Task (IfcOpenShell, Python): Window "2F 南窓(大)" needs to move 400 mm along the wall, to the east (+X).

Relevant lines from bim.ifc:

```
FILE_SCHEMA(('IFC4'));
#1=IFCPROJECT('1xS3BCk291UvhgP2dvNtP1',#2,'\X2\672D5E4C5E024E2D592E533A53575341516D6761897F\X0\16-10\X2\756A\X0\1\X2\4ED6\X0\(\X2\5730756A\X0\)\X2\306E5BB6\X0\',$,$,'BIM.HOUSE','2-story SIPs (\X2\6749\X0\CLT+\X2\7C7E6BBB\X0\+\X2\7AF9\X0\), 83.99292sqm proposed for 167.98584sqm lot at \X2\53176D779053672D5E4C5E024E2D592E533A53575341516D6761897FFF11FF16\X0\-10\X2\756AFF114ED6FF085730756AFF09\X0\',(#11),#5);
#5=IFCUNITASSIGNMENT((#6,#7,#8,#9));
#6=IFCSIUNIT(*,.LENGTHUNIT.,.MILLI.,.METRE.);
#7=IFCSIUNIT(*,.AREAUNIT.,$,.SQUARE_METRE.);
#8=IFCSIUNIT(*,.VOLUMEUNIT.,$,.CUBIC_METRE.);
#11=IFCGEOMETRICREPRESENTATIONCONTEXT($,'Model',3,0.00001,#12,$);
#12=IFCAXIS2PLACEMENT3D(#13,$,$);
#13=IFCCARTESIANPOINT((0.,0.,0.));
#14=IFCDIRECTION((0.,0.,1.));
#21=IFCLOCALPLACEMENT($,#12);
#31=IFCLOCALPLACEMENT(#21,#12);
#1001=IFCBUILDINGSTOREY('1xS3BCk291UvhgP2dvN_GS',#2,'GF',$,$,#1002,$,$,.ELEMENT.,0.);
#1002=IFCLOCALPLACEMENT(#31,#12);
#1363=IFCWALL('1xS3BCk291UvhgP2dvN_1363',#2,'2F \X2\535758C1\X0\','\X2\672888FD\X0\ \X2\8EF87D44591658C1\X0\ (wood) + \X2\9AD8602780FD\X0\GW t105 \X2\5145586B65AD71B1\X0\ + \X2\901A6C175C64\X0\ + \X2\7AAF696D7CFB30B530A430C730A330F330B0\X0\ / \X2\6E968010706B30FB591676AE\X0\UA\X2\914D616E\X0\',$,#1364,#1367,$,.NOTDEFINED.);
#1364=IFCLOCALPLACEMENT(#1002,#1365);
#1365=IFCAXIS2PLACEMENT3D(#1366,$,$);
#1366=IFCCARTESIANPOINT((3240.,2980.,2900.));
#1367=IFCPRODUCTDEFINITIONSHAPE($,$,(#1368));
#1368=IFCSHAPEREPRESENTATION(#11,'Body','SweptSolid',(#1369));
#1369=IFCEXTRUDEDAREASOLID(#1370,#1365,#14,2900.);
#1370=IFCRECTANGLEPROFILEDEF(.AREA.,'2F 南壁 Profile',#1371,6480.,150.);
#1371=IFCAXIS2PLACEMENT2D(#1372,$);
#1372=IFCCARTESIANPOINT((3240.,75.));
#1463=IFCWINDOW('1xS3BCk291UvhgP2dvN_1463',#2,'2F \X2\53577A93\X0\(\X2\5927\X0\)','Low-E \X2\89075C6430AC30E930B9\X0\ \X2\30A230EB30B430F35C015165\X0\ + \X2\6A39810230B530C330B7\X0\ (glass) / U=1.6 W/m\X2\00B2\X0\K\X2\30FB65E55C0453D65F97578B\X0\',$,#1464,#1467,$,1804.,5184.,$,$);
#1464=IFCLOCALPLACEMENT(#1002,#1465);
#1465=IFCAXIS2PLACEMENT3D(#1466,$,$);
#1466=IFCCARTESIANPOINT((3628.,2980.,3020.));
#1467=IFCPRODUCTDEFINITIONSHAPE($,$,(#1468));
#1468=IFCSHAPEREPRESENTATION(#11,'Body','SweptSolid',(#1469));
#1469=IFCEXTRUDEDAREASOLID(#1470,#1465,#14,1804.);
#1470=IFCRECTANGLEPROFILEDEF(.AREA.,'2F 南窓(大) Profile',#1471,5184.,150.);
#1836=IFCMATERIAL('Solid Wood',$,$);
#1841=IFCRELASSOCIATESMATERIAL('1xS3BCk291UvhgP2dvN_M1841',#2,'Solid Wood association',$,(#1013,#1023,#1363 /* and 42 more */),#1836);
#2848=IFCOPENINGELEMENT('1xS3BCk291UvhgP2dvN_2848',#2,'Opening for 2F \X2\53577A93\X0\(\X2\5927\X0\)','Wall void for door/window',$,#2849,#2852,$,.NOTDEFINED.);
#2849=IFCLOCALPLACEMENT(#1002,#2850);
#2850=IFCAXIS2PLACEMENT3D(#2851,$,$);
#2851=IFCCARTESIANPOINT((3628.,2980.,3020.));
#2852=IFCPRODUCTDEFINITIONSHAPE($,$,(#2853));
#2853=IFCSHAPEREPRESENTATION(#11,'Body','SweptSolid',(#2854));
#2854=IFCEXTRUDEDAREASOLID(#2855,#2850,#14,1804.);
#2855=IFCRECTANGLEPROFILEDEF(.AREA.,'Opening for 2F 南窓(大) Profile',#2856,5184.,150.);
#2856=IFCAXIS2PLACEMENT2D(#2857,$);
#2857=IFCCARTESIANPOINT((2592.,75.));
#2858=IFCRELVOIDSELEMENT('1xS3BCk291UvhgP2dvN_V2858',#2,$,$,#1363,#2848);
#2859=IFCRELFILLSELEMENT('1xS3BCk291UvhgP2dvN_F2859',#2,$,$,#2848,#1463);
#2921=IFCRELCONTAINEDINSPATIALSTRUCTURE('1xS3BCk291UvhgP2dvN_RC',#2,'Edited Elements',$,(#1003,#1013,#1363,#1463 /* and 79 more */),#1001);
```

```python
import ifcopenshell
import ifcopenshell.api.geometry
import ifcopenshell.util.placement

model = ifcopenshell.open("bim.ifc")

window = model.by_guid("1xS3BCk291UvhgP2dvN_1463")
opening = window.FillsVoids[0].RelatingOpeningElement
wall = opening.VoidsElements[0].RelatingBuildingElement

wall_matrix = ifcopenshell.util.placement.get_local_placement(wall.ObjectPlacement)
shift = wall_matrix[:3, 0] * 400.0
before = ifcopenshell.util.placement.get_local_placement(window.ObjectPlacement)[:3, 3].copy()

# The window is not placed relative to its opening, so move both.
for product in (opening, window):
    matrix = ifcopenshell.util.placement.get_local_placement(product.ObjectPlacement)
    matrix[:3, 3] += shift
    ifcopenshell.api.geometry.edit_object_placement(model, product=product, matrix=matrix, is_si=False)

after = ifcopenshell.util.placement.get_local_placement(window.ObjectPlacement)[:3, 3]
print("window moved by", (after - before).round(3) + 0.0)

model.write("bim_rev.ifc")
```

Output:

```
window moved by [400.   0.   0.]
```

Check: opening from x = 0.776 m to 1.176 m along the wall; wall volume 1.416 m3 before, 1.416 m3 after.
